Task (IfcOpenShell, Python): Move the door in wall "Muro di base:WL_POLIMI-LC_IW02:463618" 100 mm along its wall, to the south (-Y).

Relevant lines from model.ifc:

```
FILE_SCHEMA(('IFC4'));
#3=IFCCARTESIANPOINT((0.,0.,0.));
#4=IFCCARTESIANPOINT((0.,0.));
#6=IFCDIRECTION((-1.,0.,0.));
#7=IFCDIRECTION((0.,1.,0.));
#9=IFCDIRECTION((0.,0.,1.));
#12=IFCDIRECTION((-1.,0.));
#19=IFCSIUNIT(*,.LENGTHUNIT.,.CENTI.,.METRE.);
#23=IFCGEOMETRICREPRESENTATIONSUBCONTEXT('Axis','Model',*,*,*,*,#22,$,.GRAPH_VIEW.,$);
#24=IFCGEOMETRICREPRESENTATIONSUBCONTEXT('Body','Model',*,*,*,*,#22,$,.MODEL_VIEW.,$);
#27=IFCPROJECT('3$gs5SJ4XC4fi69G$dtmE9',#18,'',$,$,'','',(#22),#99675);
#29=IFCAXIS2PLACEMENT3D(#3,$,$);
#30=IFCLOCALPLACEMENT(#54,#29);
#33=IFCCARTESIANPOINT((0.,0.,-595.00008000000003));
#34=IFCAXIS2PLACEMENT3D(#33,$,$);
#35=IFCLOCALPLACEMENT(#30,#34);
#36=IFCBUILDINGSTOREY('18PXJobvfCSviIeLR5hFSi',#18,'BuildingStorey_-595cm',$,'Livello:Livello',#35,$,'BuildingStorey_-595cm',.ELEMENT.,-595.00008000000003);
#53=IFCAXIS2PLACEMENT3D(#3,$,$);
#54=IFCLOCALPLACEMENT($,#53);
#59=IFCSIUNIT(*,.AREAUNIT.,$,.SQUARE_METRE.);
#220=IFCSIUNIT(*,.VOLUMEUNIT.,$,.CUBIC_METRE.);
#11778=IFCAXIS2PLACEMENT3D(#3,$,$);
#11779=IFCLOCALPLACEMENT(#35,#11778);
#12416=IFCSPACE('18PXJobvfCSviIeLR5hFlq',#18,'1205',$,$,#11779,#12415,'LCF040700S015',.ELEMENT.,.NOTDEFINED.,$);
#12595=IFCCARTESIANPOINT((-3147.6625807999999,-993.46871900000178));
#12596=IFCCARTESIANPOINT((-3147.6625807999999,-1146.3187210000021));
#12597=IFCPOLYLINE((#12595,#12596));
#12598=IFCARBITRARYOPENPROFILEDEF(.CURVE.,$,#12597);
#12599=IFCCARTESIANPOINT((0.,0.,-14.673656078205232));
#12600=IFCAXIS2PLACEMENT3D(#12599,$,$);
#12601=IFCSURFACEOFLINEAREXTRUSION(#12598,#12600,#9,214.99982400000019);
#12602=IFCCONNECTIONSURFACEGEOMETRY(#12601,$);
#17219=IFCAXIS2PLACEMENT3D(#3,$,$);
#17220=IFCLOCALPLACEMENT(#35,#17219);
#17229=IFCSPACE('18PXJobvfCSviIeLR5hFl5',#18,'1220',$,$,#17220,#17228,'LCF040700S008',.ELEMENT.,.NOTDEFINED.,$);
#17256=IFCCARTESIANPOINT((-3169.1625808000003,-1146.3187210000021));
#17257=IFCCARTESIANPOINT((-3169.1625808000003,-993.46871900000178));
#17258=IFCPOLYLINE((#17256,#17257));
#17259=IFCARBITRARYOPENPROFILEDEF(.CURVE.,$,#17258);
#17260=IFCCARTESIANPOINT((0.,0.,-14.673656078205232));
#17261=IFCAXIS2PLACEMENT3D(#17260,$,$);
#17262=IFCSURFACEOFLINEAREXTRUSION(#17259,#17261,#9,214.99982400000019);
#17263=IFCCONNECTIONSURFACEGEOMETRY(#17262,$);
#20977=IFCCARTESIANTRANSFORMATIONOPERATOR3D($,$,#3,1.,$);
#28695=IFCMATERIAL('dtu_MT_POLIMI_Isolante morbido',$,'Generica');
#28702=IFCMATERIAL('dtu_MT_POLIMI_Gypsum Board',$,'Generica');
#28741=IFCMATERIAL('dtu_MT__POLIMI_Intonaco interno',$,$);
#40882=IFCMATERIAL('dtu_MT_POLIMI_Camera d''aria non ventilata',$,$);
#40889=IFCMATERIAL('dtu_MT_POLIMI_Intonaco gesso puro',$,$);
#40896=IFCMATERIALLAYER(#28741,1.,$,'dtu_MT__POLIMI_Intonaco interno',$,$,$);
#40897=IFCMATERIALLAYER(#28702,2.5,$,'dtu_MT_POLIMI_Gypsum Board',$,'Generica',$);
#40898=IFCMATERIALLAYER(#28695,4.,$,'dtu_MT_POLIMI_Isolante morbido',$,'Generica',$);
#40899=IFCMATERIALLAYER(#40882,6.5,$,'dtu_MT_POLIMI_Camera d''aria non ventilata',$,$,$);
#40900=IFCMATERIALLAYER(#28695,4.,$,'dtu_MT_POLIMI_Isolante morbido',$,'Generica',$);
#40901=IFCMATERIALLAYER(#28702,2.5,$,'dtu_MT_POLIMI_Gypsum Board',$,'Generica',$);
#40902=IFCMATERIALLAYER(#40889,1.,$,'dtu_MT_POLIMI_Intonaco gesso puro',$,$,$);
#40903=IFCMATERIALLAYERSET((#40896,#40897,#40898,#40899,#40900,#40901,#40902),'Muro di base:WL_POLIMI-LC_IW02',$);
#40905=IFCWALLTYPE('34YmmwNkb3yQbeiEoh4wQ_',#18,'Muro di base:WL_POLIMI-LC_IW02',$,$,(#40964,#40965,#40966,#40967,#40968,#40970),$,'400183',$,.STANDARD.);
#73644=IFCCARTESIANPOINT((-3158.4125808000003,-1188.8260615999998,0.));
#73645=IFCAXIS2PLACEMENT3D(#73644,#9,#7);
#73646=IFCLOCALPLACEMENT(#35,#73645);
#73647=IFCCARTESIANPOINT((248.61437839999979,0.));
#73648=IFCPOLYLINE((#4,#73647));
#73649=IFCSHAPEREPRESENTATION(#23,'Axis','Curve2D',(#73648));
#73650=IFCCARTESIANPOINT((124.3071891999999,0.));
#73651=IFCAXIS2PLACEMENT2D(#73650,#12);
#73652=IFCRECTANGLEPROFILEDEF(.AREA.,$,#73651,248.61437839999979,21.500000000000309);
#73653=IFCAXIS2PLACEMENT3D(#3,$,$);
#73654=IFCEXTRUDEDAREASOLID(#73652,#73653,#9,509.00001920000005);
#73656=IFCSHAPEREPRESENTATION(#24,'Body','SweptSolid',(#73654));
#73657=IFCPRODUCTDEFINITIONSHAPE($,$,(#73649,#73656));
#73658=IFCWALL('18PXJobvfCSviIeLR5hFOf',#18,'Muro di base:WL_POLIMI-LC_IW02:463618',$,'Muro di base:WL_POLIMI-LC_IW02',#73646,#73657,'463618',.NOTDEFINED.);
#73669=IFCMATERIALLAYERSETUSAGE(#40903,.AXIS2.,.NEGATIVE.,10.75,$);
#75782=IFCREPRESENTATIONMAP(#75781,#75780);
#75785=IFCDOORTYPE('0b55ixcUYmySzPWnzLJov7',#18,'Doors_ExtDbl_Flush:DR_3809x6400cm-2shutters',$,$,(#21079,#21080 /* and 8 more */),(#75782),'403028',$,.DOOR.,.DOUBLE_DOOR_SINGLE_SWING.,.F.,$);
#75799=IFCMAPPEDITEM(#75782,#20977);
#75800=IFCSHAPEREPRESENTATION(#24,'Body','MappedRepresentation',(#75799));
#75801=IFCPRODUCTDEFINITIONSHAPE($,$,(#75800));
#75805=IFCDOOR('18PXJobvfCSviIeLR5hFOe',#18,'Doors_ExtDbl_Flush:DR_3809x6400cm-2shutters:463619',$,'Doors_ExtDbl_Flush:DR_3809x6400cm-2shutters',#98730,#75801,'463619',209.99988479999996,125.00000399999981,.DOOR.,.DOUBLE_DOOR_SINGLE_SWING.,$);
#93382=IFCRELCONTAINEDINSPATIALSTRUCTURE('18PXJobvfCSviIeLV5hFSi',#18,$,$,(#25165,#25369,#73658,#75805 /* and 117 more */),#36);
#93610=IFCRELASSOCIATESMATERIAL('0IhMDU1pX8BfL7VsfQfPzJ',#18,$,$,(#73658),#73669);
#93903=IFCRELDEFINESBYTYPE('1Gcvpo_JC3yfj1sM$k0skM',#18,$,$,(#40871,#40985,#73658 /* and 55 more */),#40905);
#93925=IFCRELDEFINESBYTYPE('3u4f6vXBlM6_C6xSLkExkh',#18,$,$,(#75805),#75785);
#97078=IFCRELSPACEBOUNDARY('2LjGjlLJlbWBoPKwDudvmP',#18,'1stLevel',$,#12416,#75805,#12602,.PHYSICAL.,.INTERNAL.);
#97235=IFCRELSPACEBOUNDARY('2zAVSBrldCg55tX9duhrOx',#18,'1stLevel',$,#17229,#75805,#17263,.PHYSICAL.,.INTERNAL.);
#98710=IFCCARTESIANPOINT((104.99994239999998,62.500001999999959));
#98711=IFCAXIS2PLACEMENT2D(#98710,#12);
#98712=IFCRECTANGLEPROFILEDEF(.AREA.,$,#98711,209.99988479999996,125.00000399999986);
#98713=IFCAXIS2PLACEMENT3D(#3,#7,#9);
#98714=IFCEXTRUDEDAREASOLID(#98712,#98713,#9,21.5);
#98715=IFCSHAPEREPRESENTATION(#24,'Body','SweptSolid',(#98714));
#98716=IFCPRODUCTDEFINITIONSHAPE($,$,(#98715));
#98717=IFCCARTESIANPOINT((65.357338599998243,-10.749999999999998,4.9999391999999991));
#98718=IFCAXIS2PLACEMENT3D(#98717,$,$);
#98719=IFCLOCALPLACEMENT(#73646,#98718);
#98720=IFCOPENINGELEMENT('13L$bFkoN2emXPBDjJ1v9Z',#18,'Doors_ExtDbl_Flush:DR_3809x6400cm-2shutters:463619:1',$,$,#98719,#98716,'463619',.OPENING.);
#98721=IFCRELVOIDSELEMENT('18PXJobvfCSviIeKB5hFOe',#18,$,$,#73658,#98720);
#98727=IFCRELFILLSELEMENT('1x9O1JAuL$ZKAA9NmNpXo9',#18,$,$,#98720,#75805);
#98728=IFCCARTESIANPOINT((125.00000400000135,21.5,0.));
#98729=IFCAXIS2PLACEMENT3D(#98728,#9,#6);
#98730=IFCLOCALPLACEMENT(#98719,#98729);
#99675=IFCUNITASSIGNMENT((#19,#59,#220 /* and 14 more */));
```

```python
import numpy as np
import ifcopenshell
import ifcopenshell.api.geometry
import ifcopenshell.util.placement
import ifcopenshell.util.unit

model = ifcopenshell.open("model.ifc")
unit_scale = ifcopenshell.util.unit.calculate_unit_scale(model)

door = model.by_guid("18PXJobvfCSviIeLR5hFOe")
opening = door.FillsVoids[0].RelatingOpeningElement
wall = opening.VoidsElements[0].RelatingBuildingElement

wall_matrix = ifcopenshell.util.placement.get_local_placement(wall.ObjectPlacement)
shift = wall_matrix[:3, 0] * -0.1 / unit_scale
before = ifcopenshell.util.placement.get_local_placement(door.ObjectPlacement)[:3, 3].copy()

# The door is placed relative to its opening, so it follows when the opening moves.
matrix = ifcopenshell.util.placement.get_local_placement(opening.ObjectPlacement)
matrix[:3, 3] += shift
ifcopenshell.api.geometry.edit_object_placement(
    model, product=opening, matrix=matrix, is_si=False, should_transform_children=True
)

# Space boundary surfaces are stored in each space's coordinates; move them too.
for rel in door.ProvidesBoundaries:
    if not rel.ConnectionGeometry:
        continue
    surface = rel.ConnectionGeometry.SurfaceOnRelatingElement
    space_matrix = ifcopenshell.util.placement.get_local_placement(rel.RelatingSpace.ObjectPlacement)
    point = np.array(surface.Position.Location.Coordinates) + space_matrix[:3, :3].T @ shift
    surface.Position = model.createIfcAxis2Placement3D(
        model.createIfcCartesianPoint(point.tolist()), surface.Position.Axis, surface.Position.RefDirection
    )

after = ifcopenshell.util.placement.get_local_placement(door.ObjectPlacement)[:3, 3]
print("door moved by", (after - before).round(3) + 0.0)

model.write("model_rev.ifc")
```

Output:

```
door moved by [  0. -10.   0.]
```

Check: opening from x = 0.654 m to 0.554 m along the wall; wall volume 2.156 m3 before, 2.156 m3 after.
